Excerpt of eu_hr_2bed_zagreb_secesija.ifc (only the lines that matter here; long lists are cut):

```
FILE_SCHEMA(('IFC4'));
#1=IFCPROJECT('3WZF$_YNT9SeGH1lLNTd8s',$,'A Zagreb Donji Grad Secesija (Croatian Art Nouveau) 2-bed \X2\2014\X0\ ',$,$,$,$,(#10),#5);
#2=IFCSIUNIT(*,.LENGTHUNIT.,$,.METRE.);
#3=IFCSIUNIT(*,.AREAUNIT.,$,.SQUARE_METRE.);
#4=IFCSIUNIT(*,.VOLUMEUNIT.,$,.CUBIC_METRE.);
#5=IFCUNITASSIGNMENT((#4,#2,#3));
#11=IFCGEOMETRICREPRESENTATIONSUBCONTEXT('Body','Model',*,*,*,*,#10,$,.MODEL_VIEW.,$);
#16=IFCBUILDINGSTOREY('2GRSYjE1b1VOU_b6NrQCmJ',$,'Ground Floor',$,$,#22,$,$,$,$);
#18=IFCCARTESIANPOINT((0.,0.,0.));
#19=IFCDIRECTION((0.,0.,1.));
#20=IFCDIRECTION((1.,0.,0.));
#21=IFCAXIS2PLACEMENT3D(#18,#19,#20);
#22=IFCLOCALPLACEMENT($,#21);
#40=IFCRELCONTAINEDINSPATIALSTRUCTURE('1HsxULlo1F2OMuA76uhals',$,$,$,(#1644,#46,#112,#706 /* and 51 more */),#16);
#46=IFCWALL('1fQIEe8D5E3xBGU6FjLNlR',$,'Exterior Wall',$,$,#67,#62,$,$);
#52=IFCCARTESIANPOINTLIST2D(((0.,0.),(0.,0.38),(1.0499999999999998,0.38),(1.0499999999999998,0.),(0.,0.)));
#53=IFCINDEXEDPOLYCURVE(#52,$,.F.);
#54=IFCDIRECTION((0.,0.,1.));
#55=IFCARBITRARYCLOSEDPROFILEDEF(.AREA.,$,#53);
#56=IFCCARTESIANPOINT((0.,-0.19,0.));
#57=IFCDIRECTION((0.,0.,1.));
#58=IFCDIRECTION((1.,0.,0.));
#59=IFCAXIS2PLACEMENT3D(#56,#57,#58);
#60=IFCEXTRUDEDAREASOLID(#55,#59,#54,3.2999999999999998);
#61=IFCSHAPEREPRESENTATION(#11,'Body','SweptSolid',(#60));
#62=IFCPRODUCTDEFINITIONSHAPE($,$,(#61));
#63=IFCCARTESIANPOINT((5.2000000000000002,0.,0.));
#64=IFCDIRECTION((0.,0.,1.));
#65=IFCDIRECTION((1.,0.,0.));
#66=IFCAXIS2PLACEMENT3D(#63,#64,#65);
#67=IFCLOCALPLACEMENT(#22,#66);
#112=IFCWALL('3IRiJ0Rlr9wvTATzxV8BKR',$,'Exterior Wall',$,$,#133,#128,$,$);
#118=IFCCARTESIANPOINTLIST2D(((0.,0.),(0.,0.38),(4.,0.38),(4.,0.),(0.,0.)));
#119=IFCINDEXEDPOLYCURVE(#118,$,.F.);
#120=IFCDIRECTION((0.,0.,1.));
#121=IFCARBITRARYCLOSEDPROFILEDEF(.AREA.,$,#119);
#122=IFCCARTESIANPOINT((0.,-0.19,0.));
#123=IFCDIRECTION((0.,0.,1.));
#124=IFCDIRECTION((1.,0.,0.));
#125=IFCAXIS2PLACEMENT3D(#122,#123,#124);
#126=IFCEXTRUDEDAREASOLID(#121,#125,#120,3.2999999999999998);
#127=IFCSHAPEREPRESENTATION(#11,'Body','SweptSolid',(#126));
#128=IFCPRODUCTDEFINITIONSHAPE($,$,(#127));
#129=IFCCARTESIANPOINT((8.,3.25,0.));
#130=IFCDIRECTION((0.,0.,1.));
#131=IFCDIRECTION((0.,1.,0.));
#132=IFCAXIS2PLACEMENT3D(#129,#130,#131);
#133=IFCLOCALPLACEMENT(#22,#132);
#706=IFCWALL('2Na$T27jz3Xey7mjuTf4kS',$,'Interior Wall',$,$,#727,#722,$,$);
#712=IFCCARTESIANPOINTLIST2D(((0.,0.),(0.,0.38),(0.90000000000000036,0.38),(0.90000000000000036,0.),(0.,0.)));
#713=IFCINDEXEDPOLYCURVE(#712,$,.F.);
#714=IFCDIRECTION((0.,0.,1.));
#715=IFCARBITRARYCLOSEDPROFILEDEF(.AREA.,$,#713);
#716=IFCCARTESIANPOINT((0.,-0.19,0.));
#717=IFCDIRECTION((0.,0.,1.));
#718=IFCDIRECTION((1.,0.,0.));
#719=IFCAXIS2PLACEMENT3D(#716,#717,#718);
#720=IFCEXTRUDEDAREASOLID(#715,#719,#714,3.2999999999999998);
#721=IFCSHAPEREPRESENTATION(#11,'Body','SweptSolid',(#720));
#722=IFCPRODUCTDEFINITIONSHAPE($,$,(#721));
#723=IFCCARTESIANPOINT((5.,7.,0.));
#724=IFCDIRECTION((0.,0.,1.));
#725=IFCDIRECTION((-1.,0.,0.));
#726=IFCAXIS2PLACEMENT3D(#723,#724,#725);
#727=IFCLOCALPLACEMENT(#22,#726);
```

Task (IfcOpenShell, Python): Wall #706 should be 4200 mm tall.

```python
import ifcopenshell
import ifcopenshell.geom
import ifcopenshell.util.representation
import ifcopenshell.util.shape
import ifcopenshell.util.unit

model = ifcopenshell.open("eu_hr_2bed_zagreb_secesija.ifc")
unit_scale = ifcopenshell.util.unit.calculate_unit_scale(model)
settings = ifcopenshell.geom.settings()


def volume(element):
    """Net volume in cubic metres, openings subtracted."""
    shape = ifcopenshell.geom.create_shape(settings, element)
    return ifcopenshell.util.shape.get_volume(shape.geometry)


wall = model.by_id(706)
before = volume(wall)

body = ifcopenshell.util.representation.get_representation(wall, "Model", "Body")
solid = body.Items[0]
old_height = solid.Depth
solid.Depth = 4.2 / unit_scale
after = volume(wall)

print(f"height {old_height:g} -> {solid.Depth:g}, volume {before:.3f} -> {after:.3f} m3")

model.write("eu_hr_2bed_zagreb_secesija_v2.ifc")
```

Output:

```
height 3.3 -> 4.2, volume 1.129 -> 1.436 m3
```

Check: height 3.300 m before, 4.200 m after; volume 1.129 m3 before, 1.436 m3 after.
